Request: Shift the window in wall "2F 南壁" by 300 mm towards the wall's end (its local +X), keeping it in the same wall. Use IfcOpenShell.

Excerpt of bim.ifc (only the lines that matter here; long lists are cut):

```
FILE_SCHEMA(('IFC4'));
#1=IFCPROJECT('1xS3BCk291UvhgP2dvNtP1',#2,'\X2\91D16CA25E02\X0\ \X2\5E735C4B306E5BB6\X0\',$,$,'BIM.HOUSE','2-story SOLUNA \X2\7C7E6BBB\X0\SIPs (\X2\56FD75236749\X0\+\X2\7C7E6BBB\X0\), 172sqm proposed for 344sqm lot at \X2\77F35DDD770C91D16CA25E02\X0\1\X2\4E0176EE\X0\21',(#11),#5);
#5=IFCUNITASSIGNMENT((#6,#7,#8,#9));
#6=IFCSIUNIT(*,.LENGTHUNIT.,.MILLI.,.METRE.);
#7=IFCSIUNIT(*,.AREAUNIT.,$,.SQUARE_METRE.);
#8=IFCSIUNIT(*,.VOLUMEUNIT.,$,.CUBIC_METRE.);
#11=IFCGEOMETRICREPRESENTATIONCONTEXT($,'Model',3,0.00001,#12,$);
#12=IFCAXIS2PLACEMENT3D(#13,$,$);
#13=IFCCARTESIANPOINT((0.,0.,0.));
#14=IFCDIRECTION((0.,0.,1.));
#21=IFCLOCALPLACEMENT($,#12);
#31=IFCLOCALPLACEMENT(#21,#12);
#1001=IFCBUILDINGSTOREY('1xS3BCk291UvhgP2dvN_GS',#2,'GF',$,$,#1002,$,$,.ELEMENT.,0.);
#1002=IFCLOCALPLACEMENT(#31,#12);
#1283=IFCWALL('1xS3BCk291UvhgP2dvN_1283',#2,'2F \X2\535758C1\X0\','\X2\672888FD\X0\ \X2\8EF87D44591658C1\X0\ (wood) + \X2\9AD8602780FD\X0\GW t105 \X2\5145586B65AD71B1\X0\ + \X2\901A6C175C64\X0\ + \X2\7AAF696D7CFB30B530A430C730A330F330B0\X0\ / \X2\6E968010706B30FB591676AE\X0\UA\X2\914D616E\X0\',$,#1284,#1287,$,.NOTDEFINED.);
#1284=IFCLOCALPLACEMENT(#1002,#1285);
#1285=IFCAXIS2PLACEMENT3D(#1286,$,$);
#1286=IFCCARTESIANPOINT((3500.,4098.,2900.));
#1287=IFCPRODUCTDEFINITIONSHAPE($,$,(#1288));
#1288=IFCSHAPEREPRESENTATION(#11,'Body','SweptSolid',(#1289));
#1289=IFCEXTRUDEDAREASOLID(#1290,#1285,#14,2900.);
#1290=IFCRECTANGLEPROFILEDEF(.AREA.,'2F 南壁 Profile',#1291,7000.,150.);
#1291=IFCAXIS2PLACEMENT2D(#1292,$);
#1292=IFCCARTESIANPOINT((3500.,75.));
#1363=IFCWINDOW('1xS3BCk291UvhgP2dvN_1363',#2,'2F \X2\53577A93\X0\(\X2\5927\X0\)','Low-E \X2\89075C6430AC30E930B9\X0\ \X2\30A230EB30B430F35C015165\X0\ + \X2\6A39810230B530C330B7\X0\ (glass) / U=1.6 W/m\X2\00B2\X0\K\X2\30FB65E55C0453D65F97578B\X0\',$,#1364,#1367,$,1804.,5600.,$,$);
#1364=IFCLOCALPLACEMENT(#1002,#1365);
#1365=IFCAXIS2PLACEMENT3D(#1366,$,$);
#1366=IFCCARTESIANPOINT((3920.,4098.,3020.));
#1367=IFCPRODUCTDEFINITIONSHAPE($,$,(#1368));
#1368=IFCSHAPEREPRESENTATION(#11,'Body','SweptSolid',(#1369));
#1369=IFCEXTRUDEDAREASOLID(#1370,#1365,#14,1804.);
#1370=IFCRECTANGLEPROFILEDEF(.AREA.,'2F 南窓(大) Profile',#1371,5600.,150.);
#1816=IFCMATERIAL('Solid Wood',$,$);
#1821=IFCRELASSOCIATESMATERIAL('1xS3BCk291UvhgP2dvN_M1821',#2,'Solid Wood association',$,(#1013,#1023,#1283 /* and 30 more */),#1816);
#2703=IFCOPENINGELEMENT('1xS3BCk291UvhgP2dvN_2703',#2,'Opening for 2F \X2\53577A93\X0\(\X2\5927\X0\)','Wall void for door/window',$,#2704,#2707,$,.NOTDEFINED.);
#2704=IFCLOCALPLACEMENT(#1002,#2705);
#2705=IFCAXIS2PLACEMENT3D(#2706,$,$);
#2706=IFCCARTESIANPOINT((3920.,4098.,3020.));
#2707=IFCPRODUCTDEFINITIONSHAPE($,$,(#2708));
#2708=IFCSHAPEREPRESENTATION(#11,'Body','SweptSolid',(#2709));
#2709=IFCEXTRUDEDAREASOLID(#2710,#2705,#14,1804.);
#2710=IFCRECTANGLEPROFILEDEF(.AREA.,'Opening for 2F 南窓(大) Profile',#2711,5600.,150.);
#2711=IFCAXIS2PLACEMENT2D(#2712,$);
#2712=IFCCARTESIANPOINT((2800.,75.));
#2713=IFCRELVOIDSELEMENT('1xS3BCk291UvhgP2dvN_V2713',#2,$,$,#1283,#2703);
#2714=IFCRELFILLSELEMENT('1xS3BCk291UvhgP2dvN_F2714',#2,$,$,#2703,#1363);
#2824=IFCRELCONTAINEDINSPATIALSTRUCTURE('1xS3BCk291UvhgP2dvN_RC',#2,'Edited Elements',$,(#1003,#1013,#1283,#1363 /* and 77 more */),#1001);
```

```python
import ifcopenshell
import ifcopenshell.api.geometry
import ifcopenshell.util.placement
import ifcopenshell.util.unit

model = ifcopenshell.open("bim.ifc")
unit_scale = ifcopenshell.util.unit.calculate_unit_scale(model)

window = model.by_guid("1xS3BCk291UvhgP2dvN_1363")
opening = window.FillsVoids[0].RelatingOpeningElement
wall = opening.VoidsElements[0].RelatingBuildingElement

wall_matrix = ifcopenshell.util.placement.get_local_placement(wall.ObjectPlacement)
shift = wall_matrix[:3, 0] * 0.3 / unit_scale
before = ifcopenshell.util.placement.get_local_placement(window.ObjectPlacement)[:3, 3].copy()

# The window is not placed relative to its opening, so move both.
for product in (opening, window):
    matrix = ifcopenshell.util.placement.get_local_placement(product.ObjectPlacement)
    matrix[:3, 3] += shift
    ifcopenshell.api.geometry.edit_object_placement(model, product=product, matrix=matrix, is_si=False)

after = ifcopenshell.util.placement.get_local_placement(window.ObjectPlacement)[:3, 3]
print("window moved by", (after - before).round(3) + 0.0)

model.write("bim_rev.ifc")
```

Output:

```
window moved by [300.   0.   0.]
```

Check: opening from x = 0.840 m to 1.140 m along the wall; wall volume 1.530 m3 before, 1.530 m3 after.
